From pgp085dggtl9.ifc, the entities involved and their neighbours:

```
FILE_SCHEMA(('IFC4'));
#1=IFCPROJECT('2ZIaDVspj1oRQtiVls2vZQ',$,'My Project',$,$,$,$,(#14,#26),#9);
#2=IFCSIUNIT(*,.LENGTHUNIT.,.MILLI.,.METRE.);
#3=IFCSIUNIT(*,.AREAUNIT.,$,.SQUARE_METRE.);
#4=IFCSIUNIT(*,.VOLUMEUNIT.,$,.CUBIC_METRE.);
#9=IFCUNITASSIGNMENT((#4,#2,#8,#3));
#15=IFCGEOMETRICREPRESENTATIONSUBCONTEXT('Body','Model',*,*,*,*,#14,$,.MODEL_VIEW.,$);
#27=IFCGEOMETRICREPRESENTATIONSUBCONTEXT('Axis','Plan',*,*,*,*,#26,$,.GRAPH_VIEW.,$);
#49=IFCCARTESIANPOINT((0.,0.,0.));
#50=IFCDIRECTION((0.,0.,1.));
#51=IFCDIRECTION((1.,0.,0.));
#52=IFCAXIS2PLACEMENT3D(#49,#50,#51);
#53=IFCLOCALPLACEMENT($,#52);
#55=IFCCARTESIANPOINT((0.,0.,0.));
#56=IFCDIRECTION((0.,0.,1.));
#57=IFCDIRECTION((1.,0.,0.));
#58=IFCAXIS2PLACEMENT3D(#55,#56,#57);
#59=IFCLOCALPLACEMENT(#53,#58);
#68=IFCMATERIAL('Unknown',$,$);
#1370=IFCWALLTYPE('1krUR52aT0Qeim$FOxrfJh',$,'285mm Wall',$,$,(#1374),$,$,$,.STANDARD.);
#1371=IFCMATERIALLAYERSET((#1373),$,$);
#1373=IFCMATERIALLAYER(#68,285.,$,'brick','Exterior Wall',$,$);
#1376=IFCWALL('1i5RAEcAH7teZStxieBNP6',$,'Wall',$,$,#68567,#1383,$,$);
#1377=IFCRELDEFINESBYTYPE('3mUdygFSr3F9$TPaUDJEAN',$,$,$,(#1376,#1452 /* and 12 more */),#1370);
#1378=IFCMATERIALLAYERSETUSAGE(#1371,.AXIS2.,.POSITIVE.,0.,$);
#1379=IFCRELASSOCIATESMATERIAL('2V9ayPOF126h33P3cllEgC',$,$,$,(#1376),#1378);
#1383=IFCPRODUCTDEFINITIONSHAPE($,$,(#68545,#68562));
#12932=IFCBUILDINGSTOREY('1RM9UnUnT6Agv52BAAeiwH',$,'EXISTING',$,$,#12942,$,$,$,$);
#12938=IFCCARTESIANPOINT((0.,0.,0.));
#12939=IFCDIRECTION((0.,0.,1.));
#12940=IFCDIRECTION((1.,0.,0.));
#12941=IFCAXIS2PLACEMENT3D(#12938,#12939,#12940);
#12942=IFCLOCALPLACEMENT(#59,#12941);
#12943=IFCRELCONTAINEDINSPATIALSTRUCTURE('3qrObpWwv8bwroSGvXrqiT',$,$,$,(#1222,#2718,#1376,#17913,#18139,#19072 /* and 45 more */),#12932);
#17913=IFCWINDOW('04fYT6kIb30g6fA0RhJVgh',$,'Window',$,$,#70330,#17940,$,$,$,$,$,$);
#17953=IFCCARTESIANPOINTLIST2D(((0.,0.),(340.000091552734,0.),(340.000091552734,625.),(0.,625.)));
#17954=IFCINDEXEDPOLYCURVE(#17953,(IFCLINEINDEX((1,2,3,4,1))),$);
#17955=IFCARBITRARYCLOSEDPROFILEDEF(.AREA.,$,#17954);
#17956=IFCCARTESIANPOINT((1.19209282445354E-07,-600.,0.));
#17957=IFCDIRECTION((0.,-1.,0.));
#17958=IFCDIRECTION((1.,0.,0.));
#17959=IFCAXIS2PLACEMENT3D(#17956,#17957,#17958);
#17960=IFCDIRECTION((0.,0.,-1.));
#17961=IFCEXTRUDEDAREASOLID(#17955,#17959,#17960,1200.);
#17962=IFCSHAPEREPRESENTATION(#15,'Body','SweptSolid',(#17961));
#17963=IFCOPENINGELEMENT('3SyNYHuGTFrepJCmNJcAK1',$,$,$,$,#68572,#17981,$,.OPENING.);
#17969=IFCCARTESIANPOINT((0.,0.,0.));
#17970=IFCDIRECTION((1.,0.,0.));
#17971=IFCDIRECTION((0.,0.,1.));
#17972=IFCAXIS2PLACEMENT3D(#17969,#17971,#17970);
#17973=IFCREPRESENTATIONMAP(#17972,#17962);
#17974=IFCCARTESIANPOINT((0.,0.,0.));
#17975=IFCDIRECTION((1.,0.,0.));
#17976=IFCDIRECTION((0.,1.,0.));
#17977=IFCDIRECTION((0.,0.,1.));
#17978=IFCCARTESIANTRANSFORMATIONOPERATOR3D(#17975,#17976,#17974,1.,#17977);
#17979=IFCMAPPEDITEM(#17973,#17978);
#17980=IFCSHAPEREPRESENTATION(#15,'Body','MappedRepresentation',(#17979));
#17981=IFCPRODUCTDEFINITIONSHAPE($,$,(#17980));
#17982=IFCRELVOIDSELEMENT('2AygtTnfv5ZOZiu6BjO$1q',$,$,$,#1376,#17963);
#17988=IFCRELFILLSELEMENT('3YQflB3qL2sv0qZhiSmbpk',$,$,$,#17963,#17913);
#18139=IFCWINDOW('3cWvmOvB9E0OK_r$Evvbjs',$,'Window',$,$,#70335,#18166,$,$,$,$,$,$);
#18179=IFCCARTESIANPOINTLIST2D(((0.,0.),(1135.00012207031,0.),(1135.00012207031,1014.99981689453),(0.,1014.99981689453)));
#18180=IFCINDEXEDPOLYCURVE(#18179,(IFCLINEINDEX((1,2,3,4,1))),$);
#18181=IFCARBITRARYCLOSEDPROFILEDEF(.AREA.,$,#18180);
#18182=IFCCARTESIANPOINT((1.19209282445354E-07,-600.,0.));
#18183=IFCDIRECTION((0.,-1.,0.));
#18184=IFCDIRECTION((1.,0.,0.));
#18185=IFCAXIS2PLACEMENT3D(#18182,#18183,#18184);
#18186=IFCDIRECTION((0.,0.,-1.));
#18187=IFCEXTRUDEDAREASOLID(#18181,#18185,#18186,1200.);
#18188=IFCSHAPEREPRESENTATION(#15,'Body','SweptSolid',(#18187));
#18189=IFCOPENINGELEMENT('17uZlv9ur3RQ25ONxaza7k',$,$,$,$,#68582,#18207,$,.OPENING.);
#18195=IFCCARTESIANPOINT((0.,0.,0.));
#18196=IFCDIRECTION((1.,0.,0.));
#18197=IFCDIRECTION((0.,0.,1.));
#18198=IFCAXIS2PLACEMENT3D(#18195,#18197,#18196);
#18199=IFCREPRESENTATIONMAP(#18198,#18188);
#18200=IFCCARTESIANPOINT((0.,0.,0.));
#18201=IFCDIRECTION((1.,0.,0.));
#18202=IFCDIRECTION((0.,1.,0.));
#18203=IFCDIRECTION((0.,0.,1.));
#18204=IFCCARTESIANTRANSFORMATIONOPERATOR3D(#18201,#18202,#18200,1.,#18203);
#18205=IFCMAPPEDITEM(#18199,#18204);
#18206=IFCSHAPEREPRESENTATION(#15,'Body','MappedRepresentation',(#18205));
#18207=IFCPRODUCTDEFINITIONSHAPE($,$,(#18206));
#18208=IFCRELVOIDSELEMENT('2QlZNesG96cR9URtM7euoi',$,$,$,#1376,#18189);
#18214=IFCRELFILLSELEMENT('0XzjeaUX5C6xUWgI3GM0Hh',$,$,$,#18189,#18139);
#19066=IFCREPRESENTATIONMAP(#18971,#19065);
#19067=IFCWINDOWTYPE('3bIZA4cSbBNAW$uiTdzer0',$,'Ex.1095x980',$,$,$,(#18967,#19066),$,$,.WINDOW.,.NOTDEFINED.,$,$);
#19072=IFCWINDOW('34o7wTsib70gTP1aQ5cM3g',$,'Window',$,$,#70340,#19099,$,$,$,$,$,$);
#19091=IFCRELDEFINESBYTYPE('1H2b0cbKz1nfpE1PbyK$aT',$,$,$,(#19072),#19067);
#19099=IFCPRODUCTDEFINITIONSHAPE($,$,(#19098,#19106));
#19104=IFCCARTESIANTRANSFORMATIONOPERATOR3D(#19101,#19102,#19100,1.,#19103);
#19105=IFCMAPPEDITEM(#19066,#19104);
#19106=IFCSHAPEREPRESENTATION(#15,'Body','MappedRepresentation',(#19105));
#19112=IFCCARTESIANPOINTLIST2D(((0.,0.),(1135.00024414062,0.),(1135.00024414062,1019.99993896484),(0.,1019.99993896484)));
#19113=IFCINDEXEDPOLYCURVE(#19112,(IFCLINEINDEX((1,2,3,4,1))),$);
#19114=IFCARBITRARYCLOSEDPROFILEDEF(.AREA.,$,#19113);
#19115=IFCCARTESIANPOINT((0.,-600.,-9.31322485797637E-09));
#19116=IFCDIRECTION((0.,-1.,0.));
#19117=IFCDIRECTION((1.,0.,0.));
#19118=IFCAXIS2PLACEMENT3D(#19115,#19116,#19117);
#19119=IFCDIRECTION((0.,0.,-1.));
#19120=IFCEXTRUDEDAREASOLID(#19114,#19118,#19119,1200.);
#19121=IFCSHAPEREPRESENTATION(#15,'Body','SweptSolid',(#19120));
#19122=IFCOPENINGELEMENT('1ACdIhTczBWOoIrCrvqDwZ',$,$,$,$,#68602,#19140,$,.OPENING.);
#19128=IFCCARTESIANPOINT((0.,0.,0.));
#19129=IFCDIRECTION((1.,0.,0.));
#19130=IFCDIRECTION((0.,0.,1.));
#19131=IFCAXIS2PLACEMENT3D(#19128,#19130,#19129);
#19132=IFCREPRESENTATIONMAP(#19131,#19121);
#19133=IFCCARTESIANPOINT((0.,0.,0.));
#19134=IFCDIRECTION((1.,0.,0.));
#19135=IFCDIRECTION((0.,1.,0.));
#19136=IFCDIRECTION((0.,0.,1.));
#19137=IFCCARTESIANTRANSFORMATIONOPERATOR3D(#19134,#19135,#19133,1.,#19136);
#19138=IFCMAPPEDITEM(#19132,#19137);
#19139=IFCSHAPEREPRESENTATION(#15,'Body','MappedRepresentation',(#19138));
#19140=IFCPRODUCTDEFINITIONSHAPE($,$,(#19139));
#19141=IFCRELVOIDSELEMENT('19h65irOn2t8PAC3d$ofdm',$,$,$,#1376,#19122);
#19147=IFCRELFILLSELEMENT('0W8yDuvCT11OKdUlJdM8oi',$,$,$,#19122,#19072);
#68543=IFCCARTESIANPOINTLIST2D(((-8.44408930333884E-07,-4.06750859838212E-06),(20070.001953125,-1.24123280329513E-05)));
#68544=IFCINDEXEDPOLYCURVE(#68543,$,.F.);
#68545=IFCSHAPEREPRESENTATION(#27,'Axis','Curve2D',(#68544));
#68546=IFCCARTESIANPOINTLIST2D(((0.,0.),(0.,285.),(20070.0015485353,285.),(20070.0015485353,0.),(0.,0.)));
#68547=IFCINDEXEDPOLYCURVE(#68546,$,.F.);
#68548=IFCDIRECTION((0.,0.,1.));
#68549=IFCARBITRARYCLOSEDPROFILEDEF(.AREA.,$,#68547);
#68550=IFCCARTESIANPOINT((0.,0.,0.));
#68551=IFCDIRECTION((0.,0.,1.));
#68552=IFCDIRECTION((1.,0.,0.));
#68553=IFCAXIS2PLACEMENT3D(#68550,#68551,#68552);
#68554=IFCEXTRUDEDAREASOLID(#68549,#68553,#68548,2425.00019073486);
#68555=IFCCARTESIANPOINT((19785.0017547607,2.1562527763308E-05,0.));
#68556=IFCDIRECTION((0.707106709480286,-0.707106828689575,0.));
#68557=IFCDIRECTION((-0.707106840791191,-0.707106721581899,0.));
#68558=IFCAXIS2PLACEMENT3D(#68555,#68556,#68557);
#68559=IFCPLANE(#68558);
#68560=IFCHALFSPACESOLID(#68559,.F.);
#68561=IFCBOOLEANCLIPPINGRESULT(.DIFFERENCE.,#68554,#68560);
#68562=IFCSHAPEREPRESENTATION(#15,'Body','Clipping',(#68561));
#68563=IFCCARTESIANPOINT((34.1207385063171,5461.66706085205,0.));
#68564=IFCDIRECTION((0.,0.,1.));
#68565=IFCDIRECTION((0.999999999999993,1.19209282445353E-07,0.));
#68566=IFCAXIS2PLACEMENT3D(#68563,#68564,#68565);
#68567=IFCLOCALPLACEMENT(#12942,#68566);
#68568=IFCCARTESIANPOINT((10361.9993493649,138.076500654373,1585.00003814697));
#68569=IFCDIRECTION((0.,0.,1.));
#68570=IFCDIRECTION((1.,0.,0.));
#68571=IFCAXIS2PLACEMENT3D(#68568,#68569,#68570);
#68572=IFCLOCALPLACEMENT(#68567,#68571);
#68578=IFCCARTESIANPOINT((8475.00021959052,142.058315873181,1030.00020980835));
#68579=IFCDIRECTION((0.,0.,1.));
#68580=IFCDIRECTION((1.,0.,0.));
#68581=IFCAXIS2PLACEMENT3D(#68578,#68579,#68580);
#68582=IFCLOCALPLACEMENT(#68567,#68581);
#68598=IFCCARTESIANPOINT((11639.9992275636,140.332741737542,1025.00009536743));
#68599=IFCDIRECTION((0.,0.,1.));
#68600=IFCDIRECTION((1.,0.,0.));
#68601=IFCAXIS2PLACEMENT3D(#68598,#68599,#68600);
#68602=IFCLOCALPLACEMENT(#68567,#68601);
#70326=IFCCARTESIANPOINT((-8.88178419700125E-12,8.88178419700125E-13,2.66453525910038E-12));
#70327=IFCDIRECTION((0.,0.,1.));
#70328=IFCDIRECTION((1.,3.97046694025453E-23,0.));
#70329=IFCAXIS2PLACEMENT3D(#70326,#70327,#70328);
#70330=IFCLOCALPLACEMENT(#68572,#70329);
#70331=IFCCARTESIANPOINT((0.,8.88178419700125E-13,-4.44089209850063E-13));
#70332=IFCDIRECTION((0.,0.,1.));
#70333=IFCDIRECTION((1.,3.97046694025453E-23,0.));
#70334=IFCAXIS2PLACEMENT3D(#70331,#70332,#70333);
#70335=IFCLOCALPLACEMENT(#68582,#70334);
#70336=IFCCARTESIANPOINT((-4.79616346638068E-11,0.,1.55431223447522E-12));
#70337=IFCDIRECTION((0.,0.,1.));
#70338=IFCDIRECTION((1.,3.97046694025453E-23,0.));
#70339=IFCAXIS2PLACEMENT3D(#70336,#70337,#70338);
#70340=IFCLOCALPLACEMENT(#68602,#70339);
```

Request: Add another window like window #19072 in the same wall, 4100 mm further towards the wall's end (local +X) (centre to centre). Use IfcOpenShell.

```python
import ifcopenshell
import ifcopenshell.api.feature
import ifcopenshell.api.geometry
import ifcopenshell.api.root
import ifcopenshell.geom
import ifcopenshell.util.element
import ifcopenshell.util.placement
import ifcopenshell.util.shape

model = ifcopenshell.open("pgp085dggtl9.ifc")
settings = ifcopenshell.geom.settings()


def volume(element):
    """Net volume in cubic metres, openings subtracted."""
    shape = ifcopenshell.geom.create_shape(settings, element)
    return ifcopenshell.util.shape.get_volume(shape.geometry)


window = model.by_id(19072)
opening = window.FillsVoids[0].RelatingOpeningElement
wall = opening.VoidsElements[0].RelatingBuildingElement
before = volume(wall)
shift = ifcopenshell.util.placement.get_local_placement(wall.ObjectPlacement)[:3, 0] * 4100.0

# copy_class copies the void relationship, type, container and properties, but no geometry.
new_opening = ifcopenshell.api.root.copy_class(model, product=opening)
new_opening.Representation = ifcopenshell.util.element.copy_deep(
    model, opening.Representation, exclude=["IfcGeometricRepresentationContext", "IfcRepresentationMap"]
)
new_window = ifcopenshell.api.root.copy_class(model, product=window)
new_window.Representation = ifcopenshell.util.element.copy_deep(
    model, window.Representation, exclude=["IfcGeometricRepresentationContext", "IfcRepresentationMap"]
)
ifcopenshell.api.feature.add_filling(model, opening=new_opening, element=new_window)

for old, new in ((opening, new_opening), (window, new_window)):
    matrix = ifcopenshell.util.placement.get_local_placement(old.ObjectPlacement)
    matrix[:3, 3] += shift
    ifcopenshell.api.geometry.edit_object_placement(model, product=new, matrix=matrix, is_si=False)

after = volume(wall)

print(f"wall volume {before:.3f} -> {after:.3f} m3")

model.write("pgp085dggtl9_edited.ifc")
```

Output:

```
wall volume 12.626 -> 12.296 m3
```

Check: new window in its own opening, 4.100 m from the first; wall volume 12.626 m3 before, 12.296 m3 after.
